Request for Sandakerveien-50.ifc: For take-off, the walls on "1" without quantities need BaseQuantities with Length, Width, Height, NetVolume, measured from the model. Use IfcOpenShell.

First a look at what the model holds.

```python
import ifcopenshell
import ifcopenshell.util.element
import ifcopenshell.util.unit

model = ifcopenshell.open("Sandakerveien-50.ifc")
print(model.schema)
for unit_type in ("LENGTHUNIT", "AREAUNIT", "VOLUMEUNIT"):
    print(unit_type, ifcopenshell.util.unit.calculate_unit_scale(model, unit_type))
storey = next(s for s in model.by_type("IfcBuildingStorey") if s.Name == "1")
walls = [e for e in ifcopenshell.util.element.get_decomposition(storey) if e.is_a("IfcWall")]
for e in sorted(walls, key=lambda e: e.id()):
    print(e.id(), e.is_a(), e.Name, list(ifcopenshell.util.element.get_psets(e, qtos_only=True)), sep=" | ")
```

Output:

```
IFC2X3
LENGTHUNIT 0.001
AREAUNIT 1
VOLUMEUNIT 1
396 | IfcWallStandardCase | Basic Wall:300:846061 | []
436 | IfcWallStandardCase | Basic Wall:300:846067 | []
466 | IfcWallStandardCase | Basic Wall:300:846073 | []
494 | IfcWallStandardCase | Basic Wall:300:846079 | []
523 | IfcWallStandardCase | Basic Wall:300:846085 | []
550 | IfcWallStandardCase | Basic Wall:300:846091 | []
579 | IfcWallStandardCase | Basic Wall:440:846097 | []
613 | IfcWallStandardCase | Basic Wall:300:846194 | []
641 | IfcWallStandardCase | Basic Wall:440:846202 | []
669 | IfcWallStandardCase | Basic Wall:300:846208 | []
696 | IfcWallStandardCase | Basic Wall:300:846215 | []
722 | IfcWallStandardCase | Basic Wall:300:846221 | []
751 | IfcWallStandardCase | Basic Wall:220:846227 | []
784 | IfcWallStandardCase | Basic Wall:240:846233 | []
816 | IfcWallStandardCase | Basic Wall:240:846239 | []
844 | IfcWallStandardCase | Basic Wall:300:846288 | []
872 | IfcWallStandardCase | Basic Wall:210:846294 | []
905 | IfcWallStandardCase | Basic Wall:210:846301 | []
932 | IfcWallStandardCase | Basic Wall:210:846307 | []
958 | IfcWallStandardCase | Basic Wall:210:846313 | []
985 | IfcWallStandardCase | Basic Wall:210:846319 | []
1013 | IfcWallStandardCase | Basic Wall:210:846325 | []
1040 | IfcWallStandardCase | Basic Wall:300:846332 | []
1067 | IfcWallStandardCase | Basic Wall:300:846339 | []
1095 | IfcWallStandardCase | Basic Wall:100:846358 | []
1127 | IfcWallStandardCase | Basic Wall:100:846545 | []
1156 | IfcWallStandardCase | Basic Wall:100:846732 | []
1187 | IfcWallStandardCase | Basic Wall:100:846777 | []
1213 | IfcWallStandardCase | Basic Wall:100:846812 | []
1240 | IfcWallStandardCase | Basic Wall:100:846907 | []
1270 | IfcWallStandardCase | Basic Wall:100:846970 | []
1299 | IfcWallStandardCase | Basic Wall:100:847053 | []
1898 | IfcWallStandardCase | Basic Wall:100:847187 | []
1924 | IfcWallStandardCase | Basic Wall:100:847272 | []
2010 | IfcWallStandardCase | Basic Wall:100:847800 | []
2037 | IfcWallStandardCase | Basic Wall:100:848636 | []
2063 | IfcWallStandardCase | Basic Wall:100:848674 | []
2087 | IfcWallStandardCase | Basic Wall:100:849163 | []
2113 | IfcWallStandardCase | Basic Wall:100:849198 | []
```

```python
import ifcopenshell
import ifcopenshell.api.pset
import ifcopenshell.geom
import ifcopenshell.util.element
import ifcopenshell.util.shape
import ifcopenshell.util.unit

model = ifcopenshell.open("Sandakerveien-50.ifc")
unit_scale = ifcopenshell.util.unit.calculate_unit_scale(model)
volume_scale = ifcopenshell.util.unit.calculate_unit_scale(model, "VOLUMEUNIT")
settings = ifcopenshell.geom.settings()

storey = next(s for s in model.by_type("IfcBuildingStorey") if s.Name == "1")
walls = [e for e in ifcopenshell.util.element.get_decomposition(storey) if e.is_a("IfcWall")]

for e in sorted(walls, key=lambda e: e.id()):
    if ifcopenshell.util.element.get_psets(e, qtos_only=True, should_inherit=False):
        continue
    # Geometry comes back in metres, in the element's own axes.
    shape = ifcopenshell.geom.create_shape(settings, e)
    values = {
        "Length": ifcopenshell.util.shape.get_x(shape.geometry) / unit_scale,
        "Width": ifcopenshell.util.shape.get_y(shape.geometry) / unit_scale,
        "Height": ifcopenshell.util.shape.get_z(shape.geometry) / unit_scale,
        "NetVolume": ifcopenshell.util.shape.get_volume(shape.geometry) / volume_scale,
    }
    qto = ifcopenshell.api.pset.add_qto(model, product=e, name="BaseQuantities")
    ifcopenshell.api.pset.edit_qto(model, qto=qto, properties=values)
    print(e.id(), {k: round(v, 3) for k, v in values.items()})

model.write("Sandakerveien-50_updated.ifc")
```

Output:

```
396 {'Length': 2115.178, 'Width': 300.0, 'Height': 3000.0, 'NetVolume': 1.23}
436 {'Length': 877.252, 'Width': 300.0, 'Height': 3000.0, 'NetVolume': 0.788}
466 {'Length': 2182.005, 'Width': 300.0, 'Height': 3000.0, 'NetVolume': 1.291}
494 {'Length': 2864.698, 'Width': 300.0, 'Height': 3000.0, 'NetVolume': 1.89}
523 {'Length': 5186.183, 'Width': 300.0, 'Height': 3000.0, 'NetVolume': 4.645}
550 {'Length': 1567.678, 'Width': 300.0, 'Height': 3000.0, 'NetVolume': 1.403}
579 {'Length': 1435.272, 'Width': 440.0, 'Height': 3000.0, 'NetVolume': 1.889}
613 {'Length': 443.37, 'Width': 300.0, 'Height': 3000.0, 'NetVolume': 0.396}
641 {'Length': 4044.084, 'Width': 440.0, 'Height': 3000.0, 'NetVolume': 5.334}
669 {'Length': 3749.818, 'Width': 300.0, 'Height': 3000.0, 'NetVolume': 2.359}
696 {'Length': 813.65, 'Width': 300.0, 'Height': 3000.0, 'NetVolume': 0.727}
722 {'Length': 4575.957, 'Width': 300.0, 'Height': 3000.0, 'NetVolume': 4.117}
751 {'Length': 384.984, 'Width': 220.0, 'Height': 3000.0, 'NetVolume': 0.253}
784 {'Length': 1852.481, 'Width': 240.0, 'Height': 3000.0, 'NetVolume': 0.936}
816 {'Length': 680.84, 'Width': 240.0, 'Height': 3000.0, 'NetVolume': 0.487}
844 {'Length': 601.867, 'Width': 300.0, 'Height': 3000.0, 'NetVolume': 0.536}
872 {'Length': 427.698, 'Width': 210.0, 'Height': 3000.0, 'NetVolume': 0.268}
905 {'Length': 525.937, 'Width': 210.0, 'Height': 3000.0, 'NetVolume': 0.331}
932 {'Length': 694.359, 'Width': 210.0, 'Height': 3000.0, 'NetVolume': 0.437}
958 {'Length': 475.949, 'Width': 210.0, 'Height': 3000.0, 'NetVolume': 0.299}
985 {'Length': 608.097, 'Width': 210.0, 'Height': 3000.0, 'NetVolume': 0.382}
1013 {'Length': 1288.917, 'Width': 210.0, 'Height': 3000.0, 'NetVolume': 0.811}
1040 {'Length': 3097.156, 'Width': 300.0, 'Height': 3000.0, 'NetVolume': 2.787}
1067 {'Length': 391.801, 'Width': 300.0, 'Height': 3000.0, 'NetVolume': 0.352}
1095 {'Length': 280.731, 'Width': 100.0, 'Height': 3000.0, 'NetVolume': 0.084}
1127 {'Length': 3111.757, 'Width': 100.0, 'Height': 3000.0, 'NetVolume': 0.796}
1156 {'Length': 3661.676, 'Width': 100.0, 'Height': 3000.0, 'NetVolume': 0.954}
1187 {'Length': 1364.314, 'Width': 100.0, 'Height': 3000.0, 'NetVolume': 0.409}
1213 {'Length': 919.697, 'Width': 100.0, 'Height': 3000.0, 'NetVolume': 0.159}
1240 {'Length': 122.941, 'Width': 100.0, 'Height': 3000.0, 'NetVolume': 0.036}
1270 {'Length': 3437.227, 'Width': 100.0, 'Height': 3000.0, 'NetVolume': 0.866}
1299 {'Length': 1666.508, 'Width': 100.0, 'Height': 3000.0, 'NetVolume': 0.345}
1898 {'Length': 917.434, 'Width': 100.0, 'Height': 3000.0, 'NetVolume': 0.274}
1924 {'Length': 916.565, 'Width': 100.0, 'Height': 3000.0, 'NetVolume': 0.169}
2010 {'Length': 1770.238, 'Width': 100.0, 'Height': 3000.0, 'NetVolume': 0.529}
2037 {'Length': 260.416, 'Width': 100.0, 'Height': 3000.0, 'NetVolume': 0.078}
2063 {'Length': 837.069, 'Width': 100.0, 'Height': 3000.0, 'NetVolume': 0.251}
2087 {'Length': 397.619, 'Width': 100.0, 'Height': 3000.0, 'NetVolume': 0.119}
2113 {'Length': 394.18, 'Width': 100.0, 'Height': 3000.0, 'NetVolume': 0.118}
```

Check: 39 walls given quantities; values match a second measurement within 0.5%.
